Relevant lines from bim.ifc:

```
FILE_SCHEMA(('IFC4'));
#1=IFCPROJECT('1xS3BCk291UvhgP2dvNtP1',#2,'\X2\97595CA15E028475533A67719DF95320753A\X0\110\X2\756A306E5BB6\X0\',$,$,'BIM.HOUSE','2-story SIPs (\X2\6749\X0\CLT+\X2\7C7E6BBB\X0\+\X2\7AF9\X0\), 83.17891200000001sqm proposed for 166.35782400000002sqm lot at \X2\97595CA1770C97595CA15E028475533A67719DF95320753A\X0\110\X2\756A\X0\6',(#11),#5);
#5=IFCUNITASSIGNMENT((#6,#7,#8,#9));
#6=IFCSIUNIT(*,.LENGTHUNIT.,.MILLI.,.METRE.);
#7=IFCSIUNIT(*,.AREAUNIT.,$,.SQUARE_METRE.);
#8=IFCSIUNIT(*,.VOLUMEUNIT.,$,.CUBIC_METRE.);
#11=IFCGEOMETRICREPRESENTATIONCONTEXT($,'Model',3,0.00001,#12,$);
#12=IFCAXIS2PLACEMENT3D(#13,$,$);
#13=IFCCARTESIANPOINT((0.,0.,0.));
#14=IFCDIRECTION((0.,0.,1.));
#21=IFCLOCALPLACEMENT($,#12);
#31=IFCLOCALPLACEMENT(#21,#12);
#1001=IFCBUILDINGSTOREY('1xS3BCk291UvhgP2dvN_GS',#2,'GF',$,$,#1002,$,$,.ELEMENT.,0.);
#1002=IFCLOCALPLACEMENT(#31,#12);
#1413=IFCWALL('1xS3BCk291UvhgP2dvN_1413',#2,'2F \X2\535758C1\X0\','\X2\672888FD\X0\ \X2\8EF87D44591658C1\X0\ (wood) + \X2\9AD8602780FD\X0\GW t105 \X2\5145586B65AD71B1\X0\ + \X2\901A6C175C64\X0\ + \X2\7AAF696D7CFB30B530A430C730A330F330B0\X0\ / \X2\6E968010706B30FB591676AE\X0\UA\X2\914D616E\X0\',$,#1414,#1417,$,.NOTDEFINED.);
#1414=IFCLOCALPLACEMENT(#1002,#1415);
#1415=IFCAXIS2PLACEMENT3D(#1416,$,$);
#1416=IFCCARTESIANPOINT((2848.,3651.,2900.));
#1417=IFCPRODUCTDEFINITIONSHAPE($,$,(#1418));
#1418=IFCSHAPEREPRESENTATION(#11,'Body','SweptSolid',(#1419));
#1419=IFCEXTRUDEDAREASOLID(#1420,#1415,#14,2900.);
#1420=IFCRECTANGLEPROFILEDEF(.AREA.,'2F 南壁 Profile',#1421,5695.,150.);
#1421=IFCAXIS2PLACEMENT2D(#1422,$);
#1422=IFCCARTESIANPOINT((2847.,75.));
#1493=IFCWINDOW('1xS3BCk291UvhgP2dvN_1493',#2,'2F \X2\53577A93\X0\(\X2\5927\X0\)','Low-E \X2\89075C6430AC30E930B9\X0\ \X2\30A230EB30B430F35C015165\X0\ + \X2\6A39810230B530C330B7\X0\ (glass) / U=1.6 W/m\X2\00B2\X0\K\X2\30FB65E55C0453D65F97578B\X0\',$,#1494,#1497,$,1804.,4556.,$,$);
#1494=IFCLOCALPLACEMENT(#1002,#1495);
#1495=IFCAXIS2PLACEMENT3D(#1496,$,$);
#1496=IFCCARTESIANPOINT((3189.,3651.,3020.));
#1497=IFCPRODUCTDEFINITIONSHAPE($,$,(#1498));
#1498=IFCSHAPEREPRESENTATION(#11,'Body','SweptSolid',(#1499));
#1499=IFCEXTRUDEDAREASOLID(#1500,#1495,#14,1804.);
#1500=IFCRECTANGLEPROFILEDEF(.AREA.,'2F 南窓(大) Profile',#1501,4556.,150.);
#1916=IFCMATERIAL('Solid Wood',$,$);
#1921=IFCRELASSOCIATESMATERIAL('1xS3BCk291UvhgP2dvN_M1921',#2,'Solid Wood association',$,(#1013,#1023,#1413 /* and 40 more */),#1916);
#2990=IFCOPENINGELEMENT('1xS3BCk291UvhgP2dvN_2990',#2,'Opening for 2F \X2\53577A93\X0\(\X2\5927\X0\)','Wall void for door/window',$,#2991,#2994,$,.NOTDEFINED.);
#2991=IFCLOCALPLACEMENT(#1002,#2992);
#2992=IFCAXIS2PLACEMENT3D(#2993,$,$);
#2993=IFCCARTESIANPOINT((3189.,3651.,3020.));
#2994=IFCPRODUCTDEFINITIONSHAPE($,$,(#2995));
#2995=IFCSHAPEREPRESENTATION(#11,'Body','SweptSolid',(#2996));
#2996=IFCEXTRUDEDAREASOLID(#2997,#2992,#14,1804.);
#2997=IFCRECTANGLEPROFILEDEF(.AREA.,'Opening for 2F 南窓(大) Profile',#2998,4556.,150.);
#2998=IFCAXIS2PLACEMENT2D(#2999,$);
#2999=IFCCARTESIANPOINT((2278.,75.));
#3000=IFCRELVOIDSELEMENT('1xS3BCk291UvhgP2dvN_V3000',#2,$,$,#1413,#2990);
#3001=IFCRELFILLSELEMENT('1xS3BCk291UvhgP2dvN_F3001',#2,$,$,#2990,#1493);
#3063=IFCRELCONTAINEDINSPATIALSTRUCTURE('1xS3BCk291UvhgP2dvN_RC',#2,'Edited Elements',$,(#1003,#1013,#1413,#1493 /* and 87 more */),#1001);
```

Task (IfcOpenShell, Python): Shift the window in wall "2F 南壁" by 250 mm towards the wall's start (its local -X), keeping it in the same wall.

```python
import ifcopenshell
import ifcopenshell.api.geometry
import ifcopenshell.util.placement

model = ifcopenshell.open("bim.ifc")

window = model.by_id(1493)
opening = window.FillsVoids[0].RelatingOpeningElement
wall = opening.VoidsElements[0].RelatingBuildingElement

wall_matrix = ifcopenshell.util.placement.get_local_placement(wall.ObjectPlacement)
shift = wall_matrix[:3, 0] * -250.0
before = ifcopenshell.util.placement.get_local_placement(window.ObjectPlacement)[:3, 3].copy()

# The window is not placed relative to its opening, so move both.
for product in (opening, window):
    matrix = ifcopenshell.util.placement.get_local_placement(product.ObjectPlacement)
    matrix[:3, 3] += shift
    ifcopenshell.api.geometry.edit_object_placement(model, product=product, matrix=matrix, is_si=False)

after = ifcopenshell.util.placement.get_local_placement(window.ObjectPlacement)[:3, 3]
print("window moved by", (after - before).round(3) + 0.0)

model.write("bim_rev.ifc")
```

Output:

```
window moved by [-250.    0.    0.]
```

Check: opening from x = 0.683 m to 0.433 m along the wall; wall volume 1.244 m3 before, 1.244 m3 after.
